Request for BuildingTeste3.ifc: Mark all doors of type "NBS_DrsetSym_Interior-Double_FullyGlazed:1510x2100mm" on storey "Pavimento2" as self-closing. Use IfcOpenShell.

First a look at what the model holds.

```python
import ifcopenshell
import ifcopenshell.util.element

model = ifcopenshell.open("BuildingTeste3.ifc")
print(model.schema)
storey = next(s for s in model.by_type("IfcBuildingStorey") if s.Name == "Pavimento2")
doors = [e for e in ifcopenshell.util.element.get_decomposition(storey) if e.is_a("IfcDoor")]
seen = {}
for e in doors:
    element_type = ifcopenshell.util.element.get_type(e)
    key = (element_type.Name if element_type != e and element_type else None, ifcopenshell.util.element.get_pset(e, "Pset_DoorCommon", "SelfClosing"))
    seen[key] = seen.get(key, 0) + 1
for (name, value), count in sorted(seen.items(), key=str):
    print(count, "x", name, "|", value)
```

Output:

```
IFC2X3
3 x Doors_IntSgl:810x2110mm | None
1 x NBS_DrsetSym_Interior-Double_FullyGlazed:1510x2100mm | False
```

```python
import ifcopenshell
import ifcopenshell.api.pset
import ifcopenshell.util.element

model = ifcopenshell.open("BuildingTeste3.ifc")

storey = next(s for s in model.by_type("IfcBuildingStorey") if s.Name == "Pavimento2")
doors = [e for e in ifcopenshell.util.element.get_decomposition(storey) if e.is_a("IfcDoor")]

count = 0
for e in doors:
    element_type = ifcopenshell.util.element.get_type(e)
    if element_type in (None, e) or element_type.Name != "NBS_DrsetSym_Interior-Double_FullyGlazed:1510x2100mm":
        continue
    # add_pset returns the element's existing set when there is one.
    pset = ifcopenshell.api.pset.add_pset(model, product=e, name="Pset_DoorCommon")
    ifcopenshell.api.pset.edit_pset(model, pset=pset, properties={"SelfClosing": True})
    count += 1

print(count, "doors updated")

model.write("BuildingTeste3_rev.ifc")
```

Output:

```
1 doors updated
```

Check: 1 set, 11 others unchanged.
